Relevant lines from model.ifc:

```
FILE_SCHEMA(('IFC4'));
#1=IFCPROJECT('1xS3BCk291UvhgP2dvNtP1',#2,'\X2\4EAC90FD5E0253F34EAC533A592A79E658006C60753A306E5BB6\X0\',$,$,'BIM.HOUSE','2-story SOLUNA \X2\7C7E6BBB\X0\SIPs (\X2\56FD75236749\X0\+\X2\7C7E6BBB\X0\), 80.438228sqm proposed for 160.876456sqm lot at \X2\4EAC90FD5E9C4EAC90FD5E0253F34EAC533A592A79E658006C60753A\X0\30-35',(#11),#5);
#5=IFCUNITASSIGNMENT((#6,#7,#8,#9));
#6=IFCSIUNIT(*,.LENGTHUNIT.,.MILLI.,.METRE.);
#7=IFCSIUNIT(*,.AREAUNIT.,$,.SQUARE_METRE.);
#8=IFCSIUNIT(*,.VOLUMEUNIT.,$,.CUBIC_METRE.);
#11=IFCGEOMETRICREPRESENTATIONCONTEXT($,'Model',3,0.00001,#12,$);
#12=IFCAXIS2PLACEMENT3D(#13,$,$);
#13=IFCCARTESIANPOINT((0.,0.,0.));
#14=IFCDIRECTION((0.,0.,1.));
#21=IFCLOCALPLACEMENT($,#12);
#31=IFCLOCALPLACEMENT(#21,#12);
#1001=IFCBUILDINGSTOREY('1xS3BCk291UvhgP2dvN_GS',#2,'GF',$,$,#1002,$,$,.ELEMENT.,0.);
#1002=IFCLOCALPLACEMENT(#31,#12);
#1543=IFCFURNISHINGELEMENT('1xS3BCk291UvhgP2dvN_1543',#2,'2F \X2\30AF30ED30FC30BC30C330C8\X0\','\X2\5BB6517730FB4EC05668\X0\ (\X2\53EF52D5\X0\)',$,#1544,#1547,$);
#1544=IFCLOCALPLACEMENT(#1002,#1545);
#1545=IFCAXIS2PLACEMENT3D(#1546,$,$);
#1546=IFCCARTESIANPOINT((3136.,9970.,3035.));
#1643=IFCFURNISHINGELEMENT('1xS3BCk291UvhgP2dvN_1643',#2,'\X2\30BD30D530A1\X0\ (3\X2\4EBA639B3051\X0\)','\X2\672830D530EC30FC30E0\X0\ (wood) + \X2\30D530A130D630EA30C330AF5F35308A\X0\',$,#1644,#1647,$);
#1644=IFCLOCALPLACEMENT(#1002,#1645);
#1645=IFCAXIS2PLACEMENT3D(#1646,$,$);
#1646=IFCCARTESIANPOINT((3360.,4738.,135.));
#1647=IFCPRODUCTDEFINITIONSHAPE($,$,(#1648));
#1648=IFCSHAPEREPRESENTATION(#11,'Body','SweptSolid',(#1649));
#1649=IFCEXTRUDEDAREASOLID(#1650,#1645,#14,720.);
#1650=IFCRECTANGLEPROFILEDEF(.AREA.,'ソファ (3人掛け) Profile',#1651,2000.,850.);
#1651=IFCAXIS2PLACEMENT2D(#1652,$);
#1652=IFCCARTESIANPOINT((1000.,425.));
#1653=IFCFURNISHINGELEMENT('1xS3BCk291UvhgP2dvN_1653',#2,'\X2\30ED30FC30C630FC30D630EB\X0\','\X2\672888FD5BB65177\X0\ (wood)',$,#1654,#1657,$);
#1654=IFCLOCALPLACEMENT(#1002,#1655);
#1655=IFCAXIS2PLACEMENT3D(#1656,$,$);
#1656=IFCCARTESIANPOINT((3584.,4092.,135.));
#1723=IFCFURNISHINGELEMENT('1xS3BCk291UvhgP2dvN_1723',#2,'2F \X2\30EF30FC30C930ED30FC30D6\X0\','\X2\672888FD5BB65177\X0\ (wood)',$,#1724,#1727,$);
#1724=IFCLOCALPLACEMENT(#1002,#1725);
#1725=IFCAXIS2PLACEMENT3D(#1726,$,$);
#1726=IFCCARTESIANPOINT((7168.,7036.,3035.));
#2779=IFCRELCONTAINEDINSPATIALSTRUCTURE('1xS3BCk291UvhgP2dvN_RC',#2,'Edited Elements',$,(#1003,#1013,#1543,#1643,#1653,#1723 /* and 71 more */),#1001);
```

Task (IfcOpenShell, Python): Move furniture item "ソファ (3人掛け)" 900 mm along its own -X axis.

```python
import ifcopenshell
import ifcopenshell.api.geometry
import ifcopenshell.util.placement
import ifcopenshell.util.unit

model = ifcopenshell.open("model.ifc")
unit_scale = ifcopenshell.util.unit.calculate_unit_scale(model)

item = model.by_guid("1xS3BCk291UvhgP2dvN_1643")
matrix = ifcopenshell.util.placement.get_local_placement(item.ObjectPlacement)
matrix[:3, 3] -= matrix[:3, 0] * 0.9 / unit_scale
ifcopenshell.api.geometry.edit_object_placement(model, product=item, matrix=matrix, is_si=False)

print(ifcopenshell.util.placement.get_local_placement(item.ObjectPlacement).round(3) + 0.0)

model.write("model_v2.ifc")
```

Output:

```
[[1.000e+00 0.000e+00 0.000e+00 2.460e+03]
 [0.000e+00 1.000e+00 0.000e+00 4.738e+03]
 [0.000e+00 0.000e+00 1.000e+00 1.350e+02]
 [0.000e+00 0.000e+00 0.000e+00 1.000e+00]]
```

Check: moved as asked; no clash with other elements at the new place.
